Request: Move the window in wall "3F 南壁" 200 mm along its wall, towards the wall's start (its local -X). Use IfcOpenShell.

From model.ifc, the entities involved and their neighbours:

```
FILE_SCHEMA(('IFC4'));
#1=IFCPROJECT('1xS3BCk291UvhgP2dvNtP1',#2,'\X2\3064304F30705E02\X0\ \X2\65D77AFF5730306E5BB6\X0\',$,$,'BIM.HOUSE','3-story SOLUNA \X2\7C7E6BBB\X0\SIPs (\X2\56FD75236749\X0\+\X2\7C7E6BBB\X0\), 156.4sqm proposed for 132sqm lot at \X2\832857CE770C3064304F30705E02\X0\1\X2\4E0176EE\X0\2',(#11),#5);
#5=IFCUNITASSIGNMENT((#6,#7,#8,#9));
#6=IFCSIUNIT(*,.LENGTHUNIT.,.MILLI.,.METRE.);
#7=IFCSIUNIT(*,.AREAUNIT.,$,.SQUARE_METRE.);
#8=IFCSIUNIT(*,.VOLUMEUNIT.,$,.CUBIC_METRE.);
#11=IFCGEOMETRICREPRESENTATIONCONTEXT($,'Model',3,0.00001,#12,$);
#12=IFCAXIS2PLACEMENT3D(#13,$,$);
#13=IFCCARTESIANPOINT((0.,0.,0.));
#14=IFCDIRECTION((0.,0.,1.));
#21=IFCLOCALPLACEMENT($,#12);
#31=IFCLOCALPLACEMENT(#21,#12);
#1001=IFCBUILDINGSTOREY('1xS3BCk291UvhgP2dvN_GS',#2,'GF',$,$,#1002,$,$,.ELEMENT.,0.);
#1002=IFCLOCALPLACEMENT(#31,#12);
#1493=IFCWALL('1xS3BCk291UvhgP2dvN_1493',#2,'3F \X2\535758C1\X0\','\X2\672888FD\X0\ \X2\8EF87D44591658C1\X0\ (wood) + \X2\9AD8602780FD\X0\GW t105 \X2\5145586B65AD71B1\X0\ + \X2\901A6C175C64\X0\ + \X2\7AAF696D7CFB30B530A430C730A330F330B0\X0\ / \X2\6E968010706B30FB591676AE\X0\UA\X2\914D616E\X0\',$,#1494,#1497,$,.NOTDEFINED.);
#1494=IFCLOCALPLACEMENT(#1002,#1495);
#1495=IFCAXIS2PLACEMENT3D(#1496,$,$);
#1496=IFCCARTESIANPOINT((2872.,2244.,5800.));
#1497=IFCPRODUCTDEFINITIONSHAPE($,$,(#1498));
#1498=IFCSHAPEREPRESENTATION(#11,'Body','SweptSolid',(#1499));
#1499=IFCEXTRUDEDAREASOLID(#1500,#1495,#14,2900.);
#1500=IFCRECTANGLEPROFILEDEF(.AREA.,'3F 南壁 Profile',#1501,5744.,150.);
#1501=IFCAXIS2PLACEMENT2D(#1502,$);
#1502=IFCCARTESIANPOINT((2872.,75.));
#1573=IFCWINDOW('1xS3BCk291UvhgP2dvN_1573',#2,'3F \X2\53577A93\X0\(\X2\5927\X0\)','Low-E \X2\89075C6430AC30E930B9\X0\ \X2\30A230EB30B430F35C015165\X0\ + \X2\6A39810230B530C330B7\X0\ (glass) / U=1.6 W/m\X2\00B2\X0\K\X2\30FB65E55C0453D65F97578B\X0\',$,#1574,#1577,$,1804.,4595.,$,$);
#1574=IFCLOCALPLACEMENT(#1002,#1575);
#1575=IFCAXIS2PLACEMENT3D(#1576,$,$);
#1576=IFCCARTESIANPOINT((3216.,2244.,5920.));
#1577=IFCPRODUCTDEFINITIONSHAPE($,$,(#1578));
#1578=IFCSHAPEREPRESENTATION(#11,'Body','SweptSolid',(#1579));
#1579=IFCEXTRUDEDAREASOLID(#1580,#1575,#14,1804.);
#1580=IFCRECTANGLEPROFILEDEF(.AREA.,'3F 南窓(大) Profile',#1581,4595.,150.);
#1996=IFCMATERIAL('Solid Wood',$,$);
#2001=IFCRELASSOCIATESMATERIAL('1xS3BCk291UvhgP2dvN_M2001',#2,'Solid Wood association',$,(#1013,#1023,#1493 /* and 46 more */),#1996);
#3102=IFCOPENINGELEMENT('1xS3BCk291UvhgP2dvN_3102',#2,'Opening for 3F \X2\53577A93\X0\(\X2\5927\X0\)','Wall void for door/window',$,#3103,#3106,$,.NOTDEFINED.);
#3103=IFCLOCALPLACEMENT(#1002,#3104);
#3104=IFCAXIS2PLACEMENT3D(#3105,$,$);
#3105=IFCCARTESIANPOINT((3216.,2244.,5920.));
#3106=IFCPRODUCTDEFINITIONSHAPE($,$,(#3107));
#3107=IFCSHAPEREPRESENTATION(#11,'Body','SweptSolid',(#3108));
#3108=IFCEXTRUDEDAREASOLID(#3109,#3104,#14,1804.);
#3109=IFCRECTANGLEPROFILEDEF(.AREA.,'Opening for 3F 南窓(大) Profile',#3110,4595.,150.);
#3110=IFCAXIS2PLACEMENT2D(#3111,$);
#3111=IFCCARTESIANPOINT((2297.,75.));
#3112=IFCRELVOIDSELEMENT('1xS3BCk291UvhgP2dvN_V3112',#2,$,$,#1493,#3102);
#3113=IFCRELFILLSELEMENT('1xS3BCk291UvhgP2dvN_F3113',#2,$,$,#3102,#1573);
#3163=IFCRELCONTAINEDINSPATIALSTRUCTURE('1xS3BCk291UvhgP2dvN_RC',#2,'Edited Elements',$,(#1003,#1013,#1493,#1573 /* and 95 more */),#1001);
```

```python
import ifcopenshell
import ifcopenshell.api.geometry
import ifcopenshell.util.placement

model = ifcopenshell.open("model.ifc")

window = model.by_id(1573)
opening = window.FillsVoids[0].RelatingOpeningElement
wall = opening.VoidsElements[0].RelatingBuildingElement

wall_matrix = ifcopenshell.util.placement.get_local_placement(wall.ObjectPlacement)
shift = wall_matrix[:3, 0] * -200.0
before = ifcopenshell.util.placement.get_local_placement(window.ObjectPlacement)[:3, 3].copy()

# The window is not placed relative to its opening, so move both.
for product in (opening, window):
    matrix = ifcopenshell.util.placement.get_local_placement(product.ObjectPlacement)
    matrix[:3, 3] += shift
    ifcopenshell.api.geometry.edit_object_placement(model, product=product, matrix=matrix, is_si=False)

after = ifcopenshell.util.placement.get_local_placement(window.ObjectPlacement)[:3, 3]
print("window moved by", (after - before).round(3) + 0.0)

model.write("model_v2.ifc")
```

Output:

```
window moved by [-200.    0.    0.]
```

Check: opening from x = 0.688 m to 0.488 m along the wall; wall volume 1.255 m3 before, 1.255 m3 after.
